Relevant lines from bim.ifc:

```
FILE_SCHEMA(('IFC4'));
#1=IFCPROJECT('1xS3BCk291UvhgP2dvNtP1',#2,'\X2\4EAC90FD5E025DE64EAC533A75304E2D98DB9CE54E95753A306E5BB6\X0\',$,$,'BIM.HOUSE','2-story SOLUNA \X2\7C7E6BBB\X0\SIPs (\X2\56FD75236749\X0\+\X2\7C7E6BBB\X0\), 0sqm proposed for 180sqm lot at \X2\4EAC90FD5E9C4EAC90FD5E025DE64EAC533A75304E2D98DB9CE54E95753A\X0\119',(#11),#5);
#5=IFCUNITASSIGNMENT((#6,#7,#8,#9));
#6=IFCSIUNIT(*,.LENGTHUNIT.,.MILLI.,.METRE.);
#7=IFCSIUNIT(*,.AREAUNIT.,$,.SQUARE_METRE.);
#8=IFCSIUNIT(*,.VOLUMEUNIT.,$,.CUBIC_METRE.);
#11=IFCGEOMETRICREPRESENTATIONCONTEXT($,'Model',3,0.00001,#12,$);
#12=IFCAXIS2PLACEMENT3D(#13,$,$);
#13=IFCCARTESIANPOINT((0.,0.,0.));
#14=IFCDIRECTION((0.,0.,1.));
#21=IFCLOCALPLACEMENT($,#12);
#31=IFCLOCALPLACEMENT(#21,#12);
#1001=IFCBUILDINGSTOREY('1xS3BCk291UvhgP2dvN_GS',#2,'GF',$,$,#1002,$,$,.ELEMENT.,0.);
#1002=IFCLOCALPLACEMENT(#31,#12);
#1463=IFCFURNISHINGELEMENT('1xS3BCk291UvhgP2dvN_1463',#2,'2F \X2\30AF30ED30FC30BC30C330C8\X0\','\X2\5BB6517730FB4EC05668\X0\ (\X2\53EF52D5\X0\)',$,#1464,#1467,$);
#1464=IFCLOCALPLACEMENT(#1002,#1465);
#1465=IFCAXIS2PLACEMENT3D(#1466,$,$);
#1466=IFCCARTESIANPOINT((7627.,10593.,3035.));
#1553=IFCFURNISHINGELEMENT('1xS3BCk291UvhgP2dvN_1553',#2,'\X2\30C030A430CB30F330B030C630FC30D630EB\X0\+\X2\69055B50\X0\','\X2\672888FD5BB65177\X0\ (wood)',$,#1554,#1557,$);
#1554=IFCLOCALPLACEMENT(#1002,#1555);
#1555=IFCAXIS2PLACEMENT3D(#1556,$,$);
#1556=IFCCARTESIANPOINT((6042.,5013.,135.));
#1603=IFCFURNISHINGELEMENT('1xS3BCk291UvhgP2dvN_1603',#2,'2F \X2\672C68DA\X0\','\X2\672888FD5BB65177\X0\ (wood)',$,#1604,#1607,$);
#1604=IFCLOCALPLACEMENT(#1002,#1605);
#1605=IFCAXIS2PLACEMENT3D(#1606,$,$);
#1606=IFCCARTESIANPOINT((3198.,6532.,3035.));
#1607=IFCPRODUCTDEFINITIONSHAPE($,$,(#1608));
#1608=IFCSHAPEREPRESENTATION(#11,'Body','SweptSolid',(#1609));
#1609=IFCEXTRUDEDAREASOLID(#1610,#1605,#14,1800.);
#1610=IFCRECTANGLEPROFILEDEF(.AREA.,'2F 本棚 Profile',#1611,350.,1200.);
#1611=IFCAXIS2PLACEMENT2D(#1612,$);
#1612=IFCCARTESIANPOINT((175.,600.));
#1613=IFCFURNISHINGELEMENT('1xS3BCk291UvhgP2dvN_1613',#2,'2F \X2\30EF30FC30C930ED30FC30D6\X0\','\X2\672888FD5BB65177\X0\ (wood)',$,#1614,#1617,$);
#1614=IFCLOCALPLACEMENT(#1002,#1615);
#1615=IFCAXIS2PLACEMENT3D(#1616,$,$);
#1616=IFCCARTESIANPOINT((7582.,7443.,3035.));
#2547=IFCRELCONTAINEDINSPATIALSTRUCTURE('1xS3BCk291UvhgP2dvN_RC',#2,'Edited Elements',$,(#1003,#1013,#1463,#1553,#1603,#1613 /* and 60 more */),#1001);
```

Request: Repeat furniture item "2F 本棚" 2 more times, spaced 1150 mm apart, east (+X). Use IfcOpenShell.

```python
import numpy as np
import ifcopenshell
import ifcopenshell.api.geometry
import ifcopenshell.api.root
import ifcopenshell.util.element
import ifcopenshell.util.placement

model = ifcopenshell.open("bim.ifc")


def reuse_history(source, copy):
    """copy_class also copies each property set's owner history, people and application; keep the originals."""
    for rel in copy.IsDefinedBy:
        if rel.is_a("IfcRelDefinesByProperties") and (history := rel.RelatingPropertyDefinition.OwnerHistory):
            rel.RelatingPropertyDefinition.OwnerHistory = source.OwnerHistory
            ifcopenshell.util.element.remove_deep2(model, history)


source = model.by_guid("1xS3BCk291UvhgP2dvN_1603")
base = ifcopenshell.util.placement.get_local_placement(source.ObjectPlacement)
step = np.array([1.0, 0.0, 0.0]) * 1150.0

for i in range(1, 3):
    copy = ifcopenshell.api.root.copy_class(model, product=source)
    copy.Representation = ifcopenshell.util.element.copy_deep(
        model, source.Representation, exclude=["IfcGeometricRepresentationContext", "IfcRepresentationMap"]
    )
    reuse_history(source, copy)
    matrix = base.copy()
    matrix[:3, 3] += i * step
    print("added at", matrix[:3, 3].round(3) + 0.0)
    ifcopenshell.api.geometry.edit_object_placement(model, product=copy, matrix=matrix, is_si=False)

model.write("bim_edited.ifc")
```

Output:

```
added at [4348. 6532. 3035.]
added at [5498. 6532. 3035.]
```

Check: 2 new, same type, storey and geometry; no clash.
